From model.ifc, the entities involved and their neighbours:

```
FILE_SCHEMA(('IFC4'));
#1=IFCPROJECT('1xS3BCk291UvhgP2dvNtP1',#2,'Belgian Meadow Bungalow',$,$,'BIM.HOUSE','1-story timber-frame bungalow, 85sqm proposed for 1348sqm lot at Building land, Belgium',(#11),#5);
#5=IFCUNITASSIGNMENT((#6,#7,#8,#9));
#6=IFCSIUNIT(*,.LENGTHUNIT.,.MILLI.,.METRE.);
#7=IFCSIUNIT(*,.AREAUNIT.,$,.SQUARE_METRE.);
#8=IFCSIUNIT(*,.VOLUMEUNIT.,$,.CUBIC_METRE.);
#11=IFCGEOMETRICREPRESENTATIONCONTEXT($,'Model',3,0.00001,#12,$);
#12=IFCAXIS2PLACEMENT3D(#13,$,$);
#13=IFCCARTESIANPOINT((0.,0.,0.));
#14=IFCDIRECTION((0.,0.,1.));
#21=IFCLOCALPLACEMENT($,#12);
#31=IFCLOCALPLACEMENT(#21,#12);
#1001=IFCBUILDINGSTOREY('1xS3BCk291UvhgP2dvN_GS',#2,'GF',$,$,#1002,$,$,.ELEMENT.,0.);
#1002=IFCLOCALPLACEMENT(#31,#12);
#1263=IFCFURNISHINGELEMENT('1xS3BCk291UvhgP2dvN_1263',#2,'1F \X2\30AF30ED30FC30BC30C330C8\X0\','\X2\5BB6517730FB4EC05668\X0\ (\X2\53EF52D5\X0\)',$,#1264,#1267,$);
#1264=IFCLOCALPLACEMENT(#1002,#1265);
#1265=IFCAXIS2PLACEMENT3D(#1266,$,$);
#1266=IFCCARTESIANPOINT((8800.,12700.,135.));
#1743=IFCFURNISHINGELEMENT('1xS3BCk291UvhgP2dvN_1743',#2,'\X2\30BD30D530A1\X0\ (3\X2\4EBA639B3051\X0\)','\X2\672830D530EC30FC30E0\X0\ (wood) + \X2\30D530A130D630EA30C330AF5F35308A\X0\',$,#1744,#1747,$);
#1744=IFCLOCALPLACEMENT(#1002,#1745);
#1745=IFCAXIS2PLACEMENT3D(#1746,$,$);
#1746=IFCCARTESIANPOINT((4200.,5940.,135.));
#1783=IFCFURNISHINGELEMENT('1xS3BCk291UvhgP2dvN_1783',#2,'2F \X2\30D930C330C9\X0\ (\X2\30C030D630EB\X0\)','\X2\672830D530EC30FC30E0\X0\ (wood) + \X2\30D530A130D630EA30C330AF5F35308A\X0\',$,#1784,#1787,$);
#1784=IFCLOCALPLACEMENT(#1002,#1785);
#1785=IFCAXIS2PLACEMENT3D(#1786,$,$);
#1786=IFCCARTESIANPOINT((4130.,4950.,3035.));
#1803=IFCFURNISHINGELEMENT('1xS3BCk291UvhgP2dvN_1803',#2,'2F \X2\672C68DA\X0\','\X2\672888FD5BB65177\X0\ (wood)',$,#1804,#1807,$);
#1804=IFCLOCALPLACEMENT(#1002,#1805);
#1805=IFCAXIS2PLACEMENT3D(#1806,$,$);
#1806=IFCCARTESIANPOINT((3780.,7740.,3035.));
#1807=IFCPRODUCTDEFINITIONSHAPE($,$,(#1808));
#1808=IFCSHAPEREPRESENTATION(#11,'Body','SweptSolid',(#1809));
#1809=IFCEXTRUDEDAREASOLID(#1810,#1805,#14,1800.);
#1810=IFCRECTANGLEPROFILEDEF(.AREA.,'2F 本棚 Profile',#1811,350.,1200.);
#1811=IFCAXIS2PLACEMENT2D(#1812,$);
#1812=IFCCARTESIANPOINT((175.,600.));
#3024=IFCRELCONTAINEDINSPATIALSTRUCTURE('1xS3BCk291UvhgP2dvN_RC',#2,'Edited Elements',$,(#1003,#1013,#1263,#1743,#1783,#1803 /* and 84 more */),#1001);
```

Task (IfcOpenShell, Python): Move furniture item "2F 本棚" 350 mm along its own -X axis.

```python
import ifcopenshell
import ifcopenshell.api.geometry
import ifcopenshell.util.placement

model = ifcopenshell.open("model.ifc")

item = model.by_guid("1xS3BCk291UvhgP2dvN_1803")
matrix = ifcopenshell.util.placement.get_local_placement(item.ObjectPlacement)
matrix[:3, 3] -= matrix[:3, 0] * 350.0
ifcopenshell.api.geometry.edit_object_placement(model, product=item, matrix=matrix, is_si=False)

print(ifcopenshell.util.placement.get_local_placement(item.ObjectPlacement).round(3) + 0.0)

model.write("model_rev.ifc")
```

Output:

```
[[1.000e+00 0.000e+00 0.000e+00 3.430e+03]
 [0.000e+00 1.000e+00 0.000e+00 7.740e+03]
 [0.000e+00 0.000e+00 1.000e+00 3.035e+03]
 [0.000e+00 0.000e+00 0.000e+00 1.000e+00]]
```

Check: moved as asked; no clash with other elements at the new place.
